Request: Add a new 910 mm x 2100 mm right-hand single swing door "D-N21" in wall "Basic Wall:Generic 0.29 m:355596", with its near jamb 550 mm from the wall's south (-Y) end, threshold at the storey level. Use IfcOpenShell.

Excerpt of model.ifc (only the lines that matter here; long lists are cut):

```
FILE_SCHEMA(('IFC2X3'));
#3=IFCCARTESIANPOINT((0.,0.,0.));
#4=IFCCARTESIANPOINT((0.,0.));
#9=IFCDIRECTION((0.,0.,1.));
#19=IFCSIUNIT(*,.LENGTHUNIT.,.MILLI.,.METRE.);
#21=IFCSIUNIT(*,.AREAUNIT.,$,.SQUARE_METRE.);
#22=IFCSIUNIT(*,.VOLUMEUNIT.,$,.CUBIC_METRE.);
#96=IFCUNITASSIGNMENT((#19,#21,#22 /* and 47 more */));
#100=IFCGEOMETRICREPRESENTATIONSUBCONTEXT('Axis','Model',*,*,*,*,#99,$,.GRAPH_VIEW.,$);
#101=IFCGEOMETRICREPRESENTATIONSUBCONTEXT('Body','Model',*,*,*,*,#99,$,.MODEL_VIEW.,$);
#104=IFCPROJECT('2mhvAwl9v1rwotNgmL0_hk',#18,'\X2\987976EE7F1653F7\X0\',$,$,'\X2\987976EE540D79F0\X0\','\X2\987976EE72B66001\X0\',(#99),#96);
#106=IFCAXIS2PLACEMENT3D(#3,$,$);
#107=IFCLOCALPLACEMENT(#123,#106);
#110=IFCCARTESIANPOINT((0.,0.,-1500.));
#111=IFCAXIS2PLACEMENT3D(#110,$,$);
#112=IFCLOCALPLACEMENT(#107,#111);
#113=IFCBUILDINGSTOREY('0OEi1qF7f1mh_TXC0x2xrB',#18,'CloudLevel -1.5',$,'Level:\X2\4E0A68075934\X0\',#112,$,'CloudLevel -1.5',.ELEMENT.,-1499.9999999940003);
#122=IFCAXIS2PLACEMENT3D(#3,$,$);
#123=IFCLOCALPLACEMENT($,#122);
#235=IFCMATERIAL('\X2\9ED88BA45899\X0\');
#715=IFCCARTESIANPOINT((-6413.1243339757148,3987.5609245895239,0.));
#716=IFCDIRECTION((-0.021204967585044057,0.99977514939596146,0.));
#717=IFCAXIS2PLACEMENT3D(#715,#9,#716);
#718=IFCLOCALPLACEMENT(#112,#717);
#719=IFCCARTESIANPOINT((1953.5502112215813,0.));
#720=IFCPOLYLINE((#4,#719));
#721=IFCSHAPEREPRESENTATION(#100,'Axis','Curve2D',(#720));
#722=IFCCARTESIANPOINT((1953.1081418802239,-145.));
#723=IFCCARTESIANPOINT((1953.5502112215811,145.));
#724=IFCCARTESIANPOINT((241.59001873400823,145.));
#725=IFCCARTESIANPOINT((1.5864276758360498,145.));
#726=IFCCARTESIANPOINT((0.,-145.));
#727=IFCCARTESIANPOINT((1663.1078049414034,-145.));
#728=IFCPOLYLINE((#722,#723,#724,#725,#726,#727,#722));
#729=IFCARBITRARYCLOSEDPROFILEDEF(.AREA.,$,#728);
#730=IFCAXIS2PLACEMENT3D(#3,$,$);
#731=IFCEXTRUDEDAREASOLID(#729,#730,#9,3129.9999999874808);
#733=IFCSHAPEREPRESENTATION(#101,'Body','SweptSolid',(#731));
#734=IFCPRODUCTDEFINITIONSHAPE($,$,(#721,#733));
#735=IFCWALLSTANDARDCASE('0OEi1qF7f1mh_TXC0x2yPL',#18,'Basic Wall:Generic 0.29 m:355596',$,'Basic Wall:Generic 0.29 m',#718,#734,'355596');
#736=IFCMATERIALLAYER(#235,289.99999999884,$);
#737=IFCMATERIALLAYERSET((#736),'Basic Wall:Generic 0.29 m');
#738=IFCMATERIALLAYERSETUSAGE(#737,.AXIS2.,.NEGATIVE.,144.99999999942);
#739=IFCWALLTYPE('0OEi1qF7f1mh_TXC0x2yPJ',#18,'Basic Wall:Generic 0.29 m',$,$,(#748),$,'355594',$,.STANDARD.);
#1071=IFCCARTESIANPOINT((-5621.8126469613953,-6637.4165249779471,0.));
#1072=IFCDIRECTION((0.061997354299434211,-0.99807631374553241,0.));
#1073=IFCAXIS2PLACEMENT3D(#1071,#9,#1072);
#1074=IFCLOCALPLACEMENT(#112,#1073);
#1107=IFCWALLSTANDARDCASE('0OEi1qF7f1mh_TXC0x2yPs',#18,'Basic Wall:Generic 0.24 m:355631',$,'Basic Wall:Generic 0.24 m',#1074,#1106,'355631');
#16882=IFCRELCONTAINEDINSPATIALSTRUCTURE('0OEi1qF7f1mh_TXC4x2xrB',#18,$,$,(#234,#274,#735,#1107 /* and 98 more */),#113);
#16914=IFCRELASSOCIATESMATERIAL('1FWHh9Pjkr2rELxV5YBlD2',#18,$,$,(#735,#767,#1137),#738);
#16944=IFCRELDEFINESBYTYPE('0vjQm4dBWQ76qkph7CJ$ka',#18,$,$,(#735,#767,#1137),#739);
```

```python
import numpy as np
import ifcopenshell
import ifcopenshell.api.feature
import ifcopenshell.api.geometry
import ifcopenshell.api.root
import ifcopenshell.api.spatial
import ifcopenshell.api.type
import ifcopenshell.geom
import ifcopenshell.util.element
import ifcopenshell.util.placement
import ifcopenshell.util.representation
import ifcopenshell.util.shape
import ifcopenshell.util.unit

model = ifcopenshell.open("model.ifc")
unit_scale = ifcopenshell.util.unit.calculate_unit_scale(model)
settings = ifcopenshell.geom.settings()


def volume(element):
    """Net volume in cubic metres, openings subtracted."""
    shape = ifcopenshell.geom.create_shape(settings, element)
    return ifcopenshell.util.shape.get_volume(shape.geometry)


wall = model.by_guid("0OEi1qF7f1mh_TXC0x2yPL")
storey = ifcopenshell.util.element.get_container(wall, ifc_class="IfcBuildingStorey")
context = ifcopenshell.util.representation.get_context(model, "Model", "Body", "MODEL_VIEW")
before = volume(wall)

width, height, from_end, sill = 0.91, 2.1, 0.55, 0.0  # metres

# The wall runs along its own X axis, and the end named is its -X end.
wall_shape = ifcopenshell.geom.create_shape(settings, wall)
x, y, z = ifcopenshell.util.shape.get_vertices(wall_shape.geometry).T
start = x.min() + from_end
face, thickness = float(y.min()), float(y.max() - y.min())
wall_matrix = ifcopenshell.util.placement.get_local_placement(wall.ObjectPlacement)
level = ifcopenshell.util.placement.get_local_placement(storey.ObjectPlacement)[2, 3]


def in_wall(x, y):
    """Placement at x, y metres in the wall's axes, at sill height."""
    matrix = wall_matrix.copy()
    matrix[:, 3] = wall_matrix @ np.array([x / unit_scale, y / unit_scale, 0.0, 1.0])
    matrix[2, 3] = level + sill / unit_scale
    return matrix


# Opening: a box that overshoots both wall faces by 50 mm.
opening = ifcopenshell.api.root.create_entity(model, ifc_class="IfcOpeningElement")
box = ifcopenshell.api.geometry.add_wall_representation(
    model, context=context, length=width, height=height, thickness=thickness + 0.1
)
ifcopenshell.api.geometry.assign_representation(model, product=opening, representation=box)
ifcopenshell.api.geometry.edit_object_placement(model, product=opening, matrix=in_wall(start, face - 0.05), is_si=False)
ifcopenshell.api.feature.add_feature(model, feature=opening, element=wall)

door = ifcopenshell.api.root.create_entity(model, ifc_class="IfcDoor", name="D-N21")
door.OverallWidth, door.OverallHeight = width / unit_scale, height / unit_scale
body = ifcopenshell.api.geometry.add_door_representation(
    model,
    context=context,
    overall_width=door.OverallWidth,
    overall_height=door.OverallHeight,
    operation_type="SINGLE_SWING_RIGHT",
    lining_properties={"LiningDepth": thickness / unit_scale, "ThresholdDepth": thickness / unit_scale},
)
ifcopenshell.api.geometry.assign_representation(model, product=door, representation=body)
ifcopenshell.api.spatial.assign_container(model, products=[door], relating_structure=storey)
fills = ifcopenshell.api.feature.add_filling(model, opening=opening, element=door)
fills.OwnerHistory = door.OwnerHistory  # required in IFC2X3

# IFC2X3 keeps the operation on the door style.
style = ifcopenshell.api.root.create_entity(model, ifc_class="IfcDoorStyle", name="D-N21")
style.OperationType, style.ConstructionType = "SINGLE_SWING_RIGHT", "NOTDEFINED"
style.ParameterTakesPrecedence = style.Sizeable = False
ifcopenshell.api.type.assign_type(model, related_objects=[door], relating_type=style)

# The lining spans the wall, so the door starts at the wall face.
ifcopenshell.api.geometry.edit_object_placement(model, product=door, matrix=in_wall(start, face), is_si=False)

after = volume(wall)

print(f"wall volume {before:.3f} -> {after:.3f} m3")

model.write("model-out.ifc")
```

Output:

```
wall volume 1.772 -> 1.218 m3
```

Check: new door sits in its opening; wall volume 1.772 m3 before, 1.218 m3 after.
